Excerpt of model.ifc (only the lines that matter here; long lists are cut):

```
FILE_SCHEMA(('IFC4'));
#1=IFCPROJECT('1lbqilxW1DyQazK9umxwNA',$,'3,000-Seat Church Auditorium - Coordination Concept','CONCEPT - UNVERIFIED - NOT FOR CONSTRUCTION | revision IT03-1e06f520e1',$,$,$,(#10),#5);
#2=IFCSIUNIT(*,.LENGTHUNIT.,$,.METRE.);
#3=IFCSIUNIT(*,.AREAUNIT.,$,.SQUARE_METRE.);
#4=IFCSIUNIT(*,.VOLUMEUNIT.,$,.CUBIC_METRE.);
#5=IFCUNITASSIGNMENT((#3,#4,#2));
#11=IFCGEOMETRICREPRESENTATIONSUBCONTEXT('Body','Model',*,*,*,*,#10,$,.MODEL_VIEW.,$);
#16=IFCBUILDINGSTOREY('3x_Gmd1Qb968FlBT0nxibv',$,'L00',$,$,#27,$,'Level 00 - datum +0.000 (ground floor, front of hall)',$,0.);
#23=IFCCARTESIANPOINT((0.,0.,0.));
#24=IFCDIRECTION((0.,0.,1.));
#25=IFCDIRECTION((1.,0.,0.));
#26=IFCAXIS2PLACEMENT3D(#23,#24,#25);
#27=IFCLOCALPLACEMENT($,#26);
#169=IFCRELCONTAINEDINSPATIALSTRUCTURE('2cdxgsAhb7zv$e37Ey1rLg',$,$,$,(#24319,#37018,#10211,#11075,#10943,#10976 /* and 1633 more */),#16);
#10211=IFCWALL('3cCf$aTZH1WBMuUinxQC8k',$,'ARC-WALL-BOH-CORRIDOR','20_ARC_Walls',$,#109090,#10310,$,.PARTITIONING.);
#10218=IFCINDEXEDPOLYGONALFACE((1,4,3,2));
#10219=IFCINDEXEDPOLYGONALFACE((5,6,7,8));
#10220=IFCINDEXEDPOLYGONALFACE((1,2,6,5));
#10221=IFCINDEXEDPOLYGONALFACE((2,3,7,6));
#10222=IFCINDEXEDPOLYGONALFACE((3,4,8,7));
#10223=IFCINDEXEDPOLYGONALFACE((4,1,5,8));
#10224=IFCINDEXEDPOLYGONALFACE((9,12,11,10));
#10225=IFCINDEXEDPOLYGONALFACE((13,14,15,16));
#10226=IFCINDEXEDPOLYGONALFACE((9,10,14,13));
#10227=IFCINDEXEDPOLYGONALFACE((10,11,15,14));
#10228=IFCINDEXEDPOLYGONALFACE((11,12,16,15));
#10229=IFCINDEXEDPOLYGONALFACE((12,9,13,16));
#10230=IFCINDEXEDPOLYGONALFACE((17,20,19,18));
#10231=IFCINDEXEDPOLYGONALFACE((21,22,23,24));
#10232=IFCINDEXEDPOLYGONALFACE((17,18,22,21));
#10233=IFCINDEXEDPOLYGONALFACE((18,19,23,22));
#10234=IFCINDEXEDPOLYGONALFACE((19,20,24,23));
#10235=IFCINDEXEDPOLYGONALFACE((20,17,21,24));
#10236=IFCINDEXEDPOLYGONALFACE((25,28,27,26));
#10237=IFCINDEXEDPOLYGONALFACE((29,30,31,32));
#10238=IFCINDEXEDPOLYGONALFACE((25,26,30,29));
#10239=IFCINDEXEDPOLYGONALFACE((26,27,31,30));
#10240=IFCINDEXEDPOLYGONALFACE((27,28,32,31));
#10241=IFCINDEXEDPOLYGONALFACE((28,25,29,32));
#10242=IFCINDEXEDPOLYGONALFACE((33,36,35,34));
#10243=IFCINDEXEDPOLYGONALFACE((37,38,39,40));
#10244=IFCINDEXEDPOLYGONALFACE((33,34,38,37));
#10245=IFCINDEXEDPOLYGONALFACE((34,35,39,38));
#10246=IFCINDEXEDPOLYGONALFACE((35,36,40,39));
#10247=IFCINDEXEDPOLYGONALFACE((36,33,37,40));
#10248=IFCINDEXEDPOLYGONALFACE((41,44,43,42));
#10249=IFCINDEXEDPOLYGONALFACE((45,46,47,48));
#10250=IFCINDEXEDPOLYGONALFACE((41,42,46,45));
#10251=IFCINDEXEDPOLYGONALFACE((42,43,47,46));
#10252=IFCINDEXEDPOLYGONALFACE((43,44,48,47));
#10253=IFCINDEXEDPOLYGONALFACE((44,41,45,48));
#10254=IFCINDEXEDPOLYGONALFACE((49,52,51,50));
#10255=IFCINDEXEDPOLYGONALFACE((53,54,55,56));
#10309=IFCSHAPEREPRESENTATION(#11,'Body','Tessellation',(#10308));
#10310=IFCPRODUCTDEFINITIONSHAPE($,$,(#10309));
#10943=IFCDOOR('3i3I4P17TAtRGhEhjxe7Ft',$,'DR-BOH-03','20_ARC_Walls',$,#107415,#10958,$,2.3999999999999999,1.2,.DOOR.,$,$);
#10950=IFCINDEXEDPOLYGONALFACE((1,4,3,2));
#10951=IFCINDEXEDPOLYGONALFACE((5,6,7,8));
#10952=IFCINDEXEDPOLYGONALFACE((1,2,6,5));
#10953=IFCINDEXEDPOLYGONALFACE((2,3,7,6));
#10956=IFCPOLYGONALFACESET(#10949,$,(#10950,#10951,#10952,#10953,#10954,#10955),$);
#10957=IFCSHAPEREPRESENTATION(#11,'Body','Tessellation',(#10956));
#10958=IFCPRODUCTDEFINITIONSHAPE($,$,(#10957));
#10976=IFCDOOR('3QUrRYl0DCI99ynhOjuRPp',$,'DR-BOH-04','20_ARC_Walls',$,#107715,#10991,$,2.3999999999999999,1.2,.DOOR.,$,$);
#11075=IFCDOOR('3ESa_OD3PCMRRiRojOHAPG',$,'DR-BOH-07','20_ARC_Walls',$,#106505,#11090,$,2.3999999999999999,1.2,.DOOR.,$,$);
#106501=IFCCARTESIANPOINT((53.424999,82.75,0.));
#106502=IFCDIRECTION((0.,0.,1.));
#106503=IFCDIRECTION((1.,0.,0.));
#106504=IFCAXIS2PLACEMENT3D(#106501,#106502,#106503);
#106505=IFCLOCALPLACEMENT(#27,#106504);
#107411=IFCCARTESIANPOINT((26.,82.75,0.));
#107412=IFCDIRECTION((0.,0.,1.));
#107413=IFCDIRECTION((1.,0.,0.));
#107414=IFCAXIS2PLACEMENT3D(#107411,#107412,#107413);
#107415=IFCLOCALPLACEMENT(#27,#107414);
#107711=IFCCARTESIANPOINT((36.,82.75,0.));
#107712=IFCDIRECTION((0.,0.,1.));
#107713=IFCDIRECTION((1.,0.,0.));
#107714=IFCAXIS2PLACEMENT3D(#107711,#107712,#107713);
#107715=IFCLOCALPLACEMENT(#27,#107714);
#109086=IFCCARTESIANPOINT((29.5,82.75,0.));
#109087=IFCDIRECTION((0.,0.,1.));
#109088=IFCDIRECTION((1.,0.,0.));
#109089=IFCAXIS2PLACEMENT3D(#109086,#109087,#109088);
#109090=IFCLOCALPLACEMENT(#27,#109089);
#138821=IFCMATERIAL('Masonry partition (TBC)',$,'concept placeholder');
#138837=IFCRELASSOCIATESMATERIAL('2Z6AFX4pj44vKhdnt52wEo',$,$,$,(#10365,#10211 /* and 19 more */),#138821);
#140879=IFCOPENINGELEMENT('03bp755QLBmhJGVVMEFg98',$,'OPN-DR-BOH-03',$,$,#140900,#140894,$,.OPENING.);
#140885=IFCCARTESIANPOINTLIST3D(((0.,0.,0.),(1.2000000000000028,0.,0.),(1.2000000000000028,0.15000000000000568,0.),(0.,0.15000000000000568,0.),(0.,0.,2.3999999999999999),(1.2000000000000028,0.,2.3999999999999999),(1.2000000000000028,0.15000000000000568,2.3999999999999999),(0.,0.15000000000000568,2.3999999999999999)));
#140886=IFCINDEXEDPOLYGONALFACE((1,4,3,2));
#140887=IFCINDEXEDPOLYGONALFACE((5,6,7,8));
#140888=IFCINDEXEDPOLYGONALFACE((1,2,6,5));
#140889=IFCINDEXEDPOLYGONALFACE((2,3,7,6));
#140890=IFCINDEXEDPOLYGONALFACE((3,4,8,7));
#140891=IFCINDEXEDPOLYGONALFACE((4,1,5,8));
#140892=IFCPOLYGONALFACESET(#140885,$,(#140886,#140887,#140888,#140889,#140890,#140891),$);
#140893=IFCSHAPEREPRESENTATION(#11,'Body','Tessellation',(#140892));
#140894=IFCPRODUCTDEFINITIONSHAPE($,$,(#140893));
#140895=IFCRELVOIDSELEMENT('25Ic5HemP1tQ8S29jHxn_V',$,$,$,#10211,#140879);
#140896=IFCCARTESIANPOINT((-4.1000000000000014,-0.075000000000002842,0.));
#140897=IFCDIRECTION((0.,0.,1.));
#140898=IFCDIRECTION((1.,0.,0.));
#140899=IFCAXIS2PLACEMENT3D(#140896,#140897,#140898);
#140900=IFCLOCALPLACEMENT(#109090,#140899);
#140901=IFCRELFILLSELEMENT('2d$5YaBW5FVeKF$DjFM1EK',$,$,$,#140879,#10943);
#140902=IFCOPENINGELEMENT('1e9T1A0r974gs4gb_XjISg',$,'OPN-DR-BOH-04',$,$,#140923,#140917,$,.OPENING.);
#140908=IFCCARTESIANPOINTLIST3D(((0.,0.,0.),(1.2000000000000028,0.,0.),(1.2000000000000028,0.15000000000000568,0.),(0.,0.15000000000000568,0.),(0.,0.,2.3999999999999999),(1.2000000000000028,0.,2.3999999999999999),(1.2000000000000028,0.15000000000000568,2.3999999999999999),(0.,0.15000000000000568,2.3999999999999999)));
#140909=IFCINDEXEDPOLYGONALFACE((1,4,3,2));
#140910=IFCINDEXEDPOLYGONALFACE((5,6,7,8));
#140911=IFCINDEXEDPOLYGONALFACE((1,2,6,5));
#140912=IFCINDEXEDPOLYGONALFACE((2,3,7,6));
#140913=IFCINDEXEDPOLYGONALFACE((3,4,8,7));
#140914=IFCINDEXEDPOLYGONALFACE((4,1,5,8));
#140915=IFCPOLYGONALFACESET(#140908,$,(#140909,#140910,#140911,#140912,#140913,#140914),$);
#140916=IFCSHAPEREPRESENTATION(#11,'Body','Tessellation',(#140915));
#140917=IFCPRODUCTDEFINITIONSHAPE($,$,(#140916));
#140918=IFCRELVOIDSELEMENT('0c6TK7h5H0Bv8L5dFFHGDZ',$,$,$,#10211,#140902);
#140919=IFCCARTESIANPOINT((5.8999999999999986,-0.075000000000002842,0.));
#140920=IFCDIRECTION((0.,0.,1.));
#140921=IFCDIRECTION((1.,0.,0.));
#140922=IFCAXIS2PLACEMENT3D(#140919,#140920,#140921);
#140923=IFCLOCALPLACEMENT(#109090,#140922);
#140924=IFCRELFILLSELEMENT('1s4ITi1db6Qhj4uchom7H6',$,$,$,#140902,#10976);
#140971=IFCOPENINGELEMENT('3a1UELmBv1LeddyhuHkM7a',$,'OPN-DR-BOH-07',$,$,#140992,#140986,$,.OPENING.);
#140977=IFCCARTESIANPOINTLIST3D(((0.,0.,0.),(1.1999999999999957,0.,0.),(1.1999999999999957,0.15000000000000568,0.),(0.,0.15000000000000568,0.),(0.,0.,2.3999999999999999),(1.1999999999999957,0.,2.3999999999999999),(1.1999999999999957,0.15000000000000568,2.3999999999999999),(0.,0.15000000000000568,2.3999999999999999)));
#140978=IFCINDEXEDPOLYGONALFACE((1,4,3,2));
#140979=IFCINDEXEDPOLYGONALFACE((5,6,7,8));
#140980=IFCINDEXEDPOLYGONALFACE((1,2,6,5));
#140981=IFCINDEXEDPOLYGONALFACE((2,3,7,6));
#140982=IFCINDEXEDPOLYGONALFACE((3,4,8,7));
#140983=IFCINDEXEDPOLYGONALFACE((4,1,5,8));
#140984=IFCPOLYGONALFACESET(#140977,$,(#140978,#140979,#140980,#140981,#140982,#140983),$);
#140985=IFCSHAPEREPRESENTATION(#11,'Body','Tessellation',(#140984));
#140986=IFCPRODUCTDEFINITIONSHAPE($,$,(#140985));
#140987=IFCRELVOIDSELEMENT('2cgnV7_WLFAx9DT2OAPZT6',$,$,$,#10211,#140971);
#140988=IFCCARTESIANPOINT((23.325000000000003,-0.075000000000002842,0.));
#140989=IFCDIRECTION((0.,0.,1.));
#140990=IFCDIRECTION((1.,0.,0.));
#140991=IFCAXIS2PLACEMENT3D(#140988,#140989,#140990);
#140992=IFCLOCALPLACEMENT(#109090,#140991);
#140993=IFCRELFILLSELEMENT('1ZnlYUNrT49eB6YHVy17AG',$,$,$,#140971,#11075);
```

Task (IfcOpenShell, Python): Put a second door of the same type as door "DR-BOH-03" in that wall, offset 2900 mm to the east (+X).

```python
import ifcopenshell
import ifcopenshell.api.feature
import ifcopenshell.api.geometry
import ifcopenshell.api.root
import ifcopenshell.geom
import ifcopenshell.util.element
import ifcopenshell.util.placement
import ifcopenshell.util.shape

model = ifcopenshell.open("model.ifc")
settings = ifcopenshell.geom.settings()


def volume(element):
    """Net volume in cubic metres, openings subtracted."""
    shape = ifcopenshell.geom.create_shape(settings, element)
    return ifcopenshell.util.shape.get_volume(shape.geometry)


door = model.by_guid("3i3I4P17TAtRGhEhjxe7Ft")
opening = door.FillsVoids[0].RelatingOpeningElement
wall = opening.VoidsElements[0].RelatingBuildingElement
before = volume(wall)
shift = ifcopenshell.util.placement.get_local_placement(wall.ObjectPlacement)[:3, 0] * 2.9

# copy_class copies the void relationship, type, container and properties, but no geometry.
new_opening = ifcopenshell.api.root.copy_class(model, product=opening)
new_opening.Representation = ifcopenshell.util.element.copy_deep(
    model, opening.Representation, exclude=["IfcGeometricRepresentationContext", "IfcRepresentationMap"]
)
new_door = ifcopenshell.api.root.copy_class(model, product=door)
new_door.Representation = ifcopenshell.util.element.copy_deep(
    model, door.Representation, exclude=["IfcGeometricRepresentationContext", "IfcRepresentationMap"]
)
ifcopenshell.api.feature.add_filling(model, opening=new_opening, element=new_door)

for old, new in ((opening, new_opening), (door, new_door)):
    matrix = ifcopenshell.util.placement.get_local_placement(old.ObjectPlacement)
    matrix[:3, 3] += shift
    ifcopenshell.api.geometry.edit_object_placement(model, product=new, matrix=matrix, is_si=False)

after = volume(wall)

print(f"wall volume {before:.3f} -> {after:.3f} m3")

model.write("model_v2.ifc")
```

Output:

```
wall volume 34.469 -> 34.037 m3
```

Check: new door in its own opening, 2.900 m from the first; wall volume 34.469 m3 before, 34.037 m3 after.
